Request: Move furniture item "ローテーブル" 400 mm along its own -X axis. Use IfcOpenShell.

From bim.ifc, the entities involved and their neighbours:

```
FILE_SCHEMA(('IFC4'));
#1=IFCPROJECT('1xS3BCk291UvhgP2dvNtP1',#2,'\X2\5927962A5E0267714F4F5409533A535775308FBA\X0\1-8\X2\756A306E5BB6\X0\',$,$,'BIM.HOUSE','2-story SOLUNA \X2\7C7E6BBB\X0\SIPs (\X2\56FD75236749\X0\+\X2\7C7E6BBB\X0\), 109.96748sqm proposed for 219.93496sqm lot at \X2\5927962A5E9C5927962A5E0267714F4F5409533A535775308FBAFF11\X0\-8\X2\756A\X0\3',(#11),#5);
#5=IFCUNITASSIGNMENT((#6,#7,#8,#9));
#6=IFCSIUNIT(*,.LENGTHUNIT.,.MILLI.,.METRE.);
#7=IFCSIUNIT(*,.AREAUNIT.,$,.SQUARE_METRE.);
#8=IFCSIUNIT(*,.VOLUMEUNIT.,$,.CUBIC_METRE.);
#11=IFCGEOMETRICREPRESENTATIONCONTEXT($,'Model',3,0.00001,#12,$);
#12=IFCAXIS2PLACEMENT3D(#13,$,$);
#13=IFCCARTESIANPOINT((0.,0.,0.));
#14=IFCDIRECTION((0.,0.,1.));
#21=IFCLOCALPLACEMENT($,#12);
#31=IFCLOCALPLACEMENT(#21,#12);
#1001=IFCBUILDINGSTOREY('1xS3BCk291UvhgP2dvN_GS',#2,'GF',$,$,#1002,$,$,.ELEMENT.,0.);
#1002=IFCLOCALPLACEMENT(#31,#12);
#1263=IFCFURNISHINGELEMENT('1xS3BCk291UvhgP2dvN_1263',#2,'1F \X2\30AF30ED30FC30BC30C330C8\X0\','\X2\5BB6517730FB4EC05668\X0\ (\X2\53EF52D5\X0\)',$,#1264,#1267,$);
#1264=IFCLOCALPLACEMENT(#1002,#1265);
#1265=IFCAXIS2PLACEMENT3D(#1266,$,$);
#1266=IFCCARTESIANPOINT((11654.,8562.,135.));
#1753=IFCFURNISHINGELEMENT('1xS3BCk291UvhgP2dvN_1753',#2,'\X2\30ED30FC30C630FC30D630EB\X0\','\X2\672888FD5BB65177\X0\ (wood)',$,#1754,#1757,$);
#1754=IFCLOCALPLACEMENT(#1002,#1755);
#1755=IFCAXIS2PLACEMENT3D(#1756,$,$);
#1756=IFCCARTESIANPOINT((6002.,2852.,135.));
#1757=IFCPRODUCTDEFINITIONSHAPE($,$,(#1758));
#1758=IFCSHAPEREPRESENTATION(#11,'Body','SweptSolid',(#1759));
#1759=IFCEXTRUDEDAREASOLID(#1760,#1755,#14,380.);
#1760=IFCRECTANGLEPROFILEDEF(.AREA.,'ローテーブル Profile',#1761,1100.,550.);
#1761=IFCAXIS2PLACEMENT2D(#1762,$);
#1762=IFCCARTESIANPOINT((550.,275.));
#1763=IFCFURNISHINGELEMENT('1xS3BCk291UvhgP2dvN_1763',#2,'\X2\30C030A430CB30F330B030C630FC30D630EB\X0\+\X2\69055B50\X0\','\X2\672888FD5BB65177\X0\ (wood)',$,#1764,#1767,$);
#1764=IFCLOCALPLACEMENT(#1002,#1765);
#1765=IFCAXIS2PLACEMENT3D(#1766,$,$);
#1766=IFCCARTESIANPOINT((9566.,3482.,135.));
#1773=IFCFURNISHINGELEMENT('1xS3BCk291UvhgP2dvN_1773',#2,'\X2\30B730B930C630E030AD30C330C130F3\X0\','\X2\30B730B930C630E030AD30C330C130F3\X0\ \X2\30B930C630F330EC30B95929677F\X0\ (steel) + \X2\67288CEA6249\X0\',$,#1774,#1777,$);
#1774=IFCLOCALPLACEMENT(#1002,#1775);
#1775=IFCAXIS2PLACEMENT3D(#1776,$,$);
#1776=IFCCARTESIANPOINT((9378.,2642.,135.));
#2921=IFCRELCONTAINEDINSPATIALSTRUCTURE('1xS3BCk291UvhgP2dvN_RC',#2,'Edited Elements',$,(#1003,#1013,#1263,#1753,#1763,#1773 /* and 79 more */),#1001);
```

```python
import ifcopenshell
import ifcopenshell.api.geometry
import ifcopenshell.util.placement

model = ifcopenshell.open("bim.ifc")

item = model.by_id(1753)
matrix = ifcopenshell.util.placement.get_local_placement(item.ObjectPlacement)
matrix[:3, 3] -= matrix[:3, 0] * 400.0
ifcopenshell.api.geometry.edit_object_placement(model, product=item, matrix=matrix, is_si=False)

print(ifcopenshell.util.placement.get_local_placement(item.ObjectPlacement).round(3) + 0.0)

model.write("bim_rev.ifc")
```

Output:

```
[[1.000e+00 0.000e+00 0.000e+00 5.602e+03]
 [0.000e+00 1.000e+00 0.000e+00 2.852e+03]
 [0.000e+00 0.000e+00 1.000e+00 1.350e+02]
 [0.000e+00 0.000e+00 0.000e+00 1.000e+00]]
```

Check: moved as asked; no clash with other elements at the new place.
